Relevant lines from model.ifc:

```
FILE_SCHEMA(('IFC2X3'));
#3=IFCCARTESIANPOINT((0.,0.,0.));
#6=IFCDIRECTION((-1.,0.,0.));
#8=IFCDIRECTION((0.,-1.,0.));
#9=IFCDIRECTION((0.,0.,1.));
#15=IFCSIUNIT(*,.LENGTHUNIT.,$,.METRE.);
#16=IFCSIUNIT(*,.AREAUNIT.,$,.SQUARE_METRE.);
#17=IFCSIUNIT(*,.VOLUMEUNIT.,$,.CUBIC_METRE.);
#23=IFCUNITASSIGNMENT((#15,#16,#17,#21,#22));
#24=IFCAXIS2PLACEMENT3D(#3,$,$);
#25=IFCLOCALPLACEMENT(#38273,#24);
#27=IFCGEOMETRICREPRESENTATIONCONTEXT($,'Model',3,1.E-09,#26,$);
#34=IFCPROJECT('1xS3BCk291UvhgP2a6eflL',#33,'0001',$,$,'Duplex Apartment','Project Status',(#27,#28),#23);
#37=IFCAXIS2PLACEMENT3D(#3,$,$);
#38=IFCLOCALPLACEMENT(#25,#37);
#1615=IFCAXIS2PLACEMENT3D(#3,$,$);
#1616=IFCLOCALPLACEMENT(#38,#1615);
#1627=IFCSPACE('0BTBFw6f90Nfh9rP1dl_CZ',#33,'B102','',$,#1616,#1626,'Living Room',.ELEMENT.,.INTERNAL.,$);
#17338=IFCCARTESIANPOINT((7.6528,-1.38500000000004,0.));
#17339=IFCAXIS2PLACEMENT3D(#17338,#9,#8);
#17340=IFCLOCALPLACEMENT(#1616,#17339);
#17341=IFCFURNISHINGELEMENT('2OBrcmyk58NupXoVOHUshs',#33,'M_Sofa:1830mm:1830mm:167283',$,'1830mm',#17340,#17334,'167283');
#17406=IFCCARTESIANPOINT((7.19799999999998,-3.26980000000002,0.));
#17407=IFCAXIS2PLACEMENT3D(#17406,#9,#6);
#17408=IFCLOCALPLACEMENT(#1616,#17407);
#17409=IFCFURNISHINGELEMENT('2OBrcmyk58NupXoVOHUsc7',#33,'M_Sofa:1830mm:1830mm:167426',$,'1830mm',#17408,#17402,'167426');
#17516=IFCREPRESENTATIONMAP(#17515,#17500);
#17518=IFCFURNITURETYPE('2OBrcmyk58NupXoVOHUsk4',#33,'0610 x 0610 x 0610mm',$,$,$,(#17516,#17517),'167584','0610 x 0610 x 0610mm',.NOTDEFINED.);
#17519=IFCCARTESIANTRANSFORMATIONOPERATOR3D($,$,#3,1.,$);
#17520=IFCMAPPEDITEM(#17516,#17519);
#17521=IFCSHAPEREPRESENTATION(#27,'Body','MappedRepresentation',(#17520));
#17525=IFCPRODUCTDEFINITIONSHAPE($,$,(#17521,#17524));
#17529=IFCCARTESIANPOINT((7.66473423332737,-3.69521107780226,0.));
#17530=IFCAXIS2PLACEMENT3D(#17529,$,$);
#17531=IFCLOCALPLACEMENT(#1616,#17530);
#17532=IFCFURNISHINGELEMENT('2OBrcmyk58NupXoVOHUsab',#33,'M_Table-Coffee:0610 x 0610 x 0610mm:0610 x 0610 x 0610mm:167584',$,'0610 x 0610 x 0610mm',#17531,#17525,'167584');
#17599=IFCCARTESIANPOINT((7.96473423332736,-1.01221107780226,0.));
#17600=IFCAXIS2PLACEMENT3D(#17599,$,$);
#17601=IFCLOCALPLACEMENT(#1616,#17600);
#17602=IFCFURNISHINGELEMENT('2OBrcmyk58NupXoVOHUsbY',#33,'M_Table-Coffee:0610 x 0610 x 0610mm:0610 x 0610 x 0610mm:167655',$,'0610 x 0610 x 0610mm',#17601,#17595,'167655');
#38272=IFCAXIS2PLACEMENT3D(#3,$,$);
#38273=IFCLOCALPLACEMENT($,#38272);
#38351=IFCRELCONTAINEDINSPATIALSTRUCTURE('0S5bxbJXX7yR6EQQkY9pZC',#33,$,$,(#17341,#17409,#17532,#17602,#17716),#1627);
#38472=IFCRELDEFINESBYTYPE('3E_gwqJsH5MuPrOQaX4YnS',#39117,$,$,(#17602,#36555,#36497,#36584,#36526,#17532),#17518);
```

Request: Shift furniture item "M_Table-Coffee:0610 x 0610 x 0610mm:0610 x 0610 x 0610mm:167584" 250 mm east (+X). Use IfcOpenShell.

```python
import ifcopenshell
import ifcopenshell.api.geometry
import ifcopenshell.util.placement

model = ifcopenshell.open("model.ifc")

item = model.by_guid("2OBrcmyk58NupXoVOHUsab")
matrix = ifcopenshell.util.placement.get_local_placement(item.ObjectPlacement)
matrix[0, 3] += 0.25
ifcopenshell.api.geometry.edit_object_placement(model, product=item, matrix=matrix, is_si=False)

print(ifcopenshell.util.placement.get_local_placement(item.ObjectPlacement).round(3) + 0.0)

model.write("model_updated.ifc")
```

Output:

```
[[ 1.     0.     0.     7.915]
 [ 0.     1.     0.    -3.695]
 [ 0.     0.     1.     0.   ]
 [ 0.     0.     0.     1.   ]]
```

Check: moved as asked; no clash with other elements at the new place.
